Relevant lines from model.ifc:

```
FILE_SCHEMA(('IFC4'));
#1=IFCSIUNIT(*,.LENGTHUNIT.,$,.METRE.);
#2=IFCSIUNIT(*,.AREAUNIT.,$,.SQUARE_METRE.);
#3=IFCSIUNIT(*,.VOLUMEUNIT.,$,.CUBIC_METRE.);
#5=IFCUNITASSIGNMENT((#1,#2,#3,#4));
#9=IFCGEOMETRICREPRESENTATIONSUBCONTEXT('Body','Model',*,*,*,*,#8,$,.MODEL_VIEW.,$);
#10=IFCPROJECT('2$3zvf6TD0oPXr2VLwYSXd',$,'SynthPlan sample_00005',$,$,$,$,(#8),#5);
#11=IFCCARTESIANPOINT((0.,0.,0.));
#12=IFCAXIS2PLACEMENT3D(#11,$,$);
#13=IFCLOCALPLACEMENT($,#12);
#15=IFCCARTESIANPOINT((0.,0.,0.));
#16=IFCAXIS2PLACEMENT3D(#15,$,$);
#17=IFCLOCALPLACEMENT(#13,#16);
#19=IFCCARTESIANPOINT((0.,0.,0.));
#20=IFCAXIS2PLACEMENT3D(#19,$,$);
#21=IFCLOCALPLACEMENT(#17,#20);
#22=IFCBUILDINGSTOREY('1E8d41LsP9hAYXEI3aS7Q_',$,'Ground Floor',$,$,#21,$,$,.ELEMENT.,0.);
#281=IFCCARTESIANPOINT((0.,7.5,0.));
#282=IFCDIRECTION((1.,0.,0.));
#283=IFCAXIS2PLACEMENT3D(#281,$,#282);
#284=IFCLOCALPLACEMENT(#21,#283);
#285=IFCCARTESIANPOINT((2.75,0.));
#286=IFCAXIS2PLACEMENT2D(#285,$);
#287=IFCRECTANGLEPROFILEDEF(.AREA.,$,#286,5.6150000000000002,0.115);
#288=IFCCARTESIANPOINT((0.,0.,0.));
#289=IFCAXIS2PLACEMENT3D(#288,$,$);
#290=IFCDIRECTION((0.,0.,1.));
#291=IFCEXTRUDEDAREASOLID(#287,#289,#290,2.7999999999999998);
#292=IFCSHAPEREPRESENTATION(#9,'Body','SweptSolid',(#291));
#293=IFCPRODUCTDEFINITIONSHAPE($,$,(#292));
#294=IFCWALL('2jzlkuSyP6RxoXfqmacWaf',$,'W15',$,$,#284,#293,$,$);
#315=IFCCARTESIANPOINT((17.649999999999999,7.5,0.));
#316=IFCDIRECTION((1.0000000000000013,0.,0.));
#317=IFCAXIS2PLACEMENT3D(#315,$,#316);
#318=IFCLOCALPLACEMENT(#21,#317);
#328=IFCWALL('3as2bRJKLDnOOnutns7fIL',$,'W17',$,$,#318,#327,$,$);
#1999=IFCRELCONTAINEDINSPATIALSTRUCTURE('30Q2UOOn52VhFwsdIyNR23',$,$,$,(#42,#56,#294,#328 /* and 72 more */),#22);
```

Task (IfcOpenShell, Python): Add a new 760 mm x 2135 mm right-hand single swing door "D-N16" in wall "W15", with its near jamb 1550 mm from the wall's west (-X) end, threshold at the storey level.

```python
import numpy as np
import ifcopenshell
import ifcopenshell.api.feature
import ifcopenshell.api.geometry
import ifcopenshell.api.root
import ifcopenshell.api.spatial
import ifcopenshell.geom
import ifcopenshell.util.element
import ifcopenshell.util.placement
import ifcopenshell.util.representation
import ifcopenshell.util.shape
import ifcopenshell.util.unit

model = ifcopenshell.open("model.ifc")
unit_scale = ifcopenshell.util.unit.calculate_unit_scale(model)
settings = ifcopenshell.geom.settings()


def volume(element):
    """Net volume in cubic metres, openings subtracted."""
    shape = ifcopenshell.geom.create_shape(settings, element)
    return ifcopenshell.util.shape.get_volume(shape.geometry)


wall = model.by_guid("2jzlkuSyP6RxoXfqmacWaf")
storey = ifcopenshell.util.element.get_container(wall, ifc_class="IfcBuildingStorey")
context = ifcopenshell.util.representation.get_context(model, "Model", "Body", "MODEL_VIEW")
before = volume(wall)

width, height, from_end, sill = 0.76, 2.135, 1.55, 0.0  # metres

# The wall runs along its own X axis, and the end named is its -X end.
wall_shape = ifcopenshell.geom.create_shape(settings, wall)
x, y, z = ifcopenshell.util.shape.get_vertices(wall_shape.geometry).T
start = x.min() + from_end
face, thickness = float(y.min()), float(y.max() - y.min())
wall_matrix = ifcopenshell.util.placement.get_local_placement(wall.ObjectPlacement)
level = ifcopenshell.util.placement.get_local_placement(storey.ObjectPlacement)[2, 3]


def in_wall(x, y):
    """Placement at x, y metres in the wall's axes, at sill height."""
    matrix = wall_matrix.copy()
    matrix[:, 3] = wall_matrix @ np.array([x / unit_scale, y / unit_scale, 0.0, 1.0])
    matrix[2, 3] = level + sill / unit_scale
    return matrix


# Opening: a box that overshoots both wall faces by 50 mm.
opening = ifcopenshell.api.root.create_entity(model, ifc_class="IfcOpeningElement", predefined_type="OPENING")
box = ifcopenshell.api.geometry.add_wall_representation(
    model, context=context, length=width, height=height, thickness=thickness + 0.1
)
ifcopenshell.api.geometry.assign_representation(model, product=opening, representation=box)
ifcopenshell.api.geometry.edit_object_placement(model, product=opening, matrix=in_wall(start, face - 0.05), is_si=False)
ifcopenshell.api.feature.add_feature(model, feature=opening, element=wall)

door = ifcopenshell.api.root.create_entity(model, ifc_class="IfcDoor", name="D-N16", predefined_type="DOOR")
door.OverallWidth, door.OverallHeight = width / unit_scale, height / unit_scale
door.OperationType = "SINGLE_SWING_RIGHT"
body = ifcopenshell.api.geometry.add_door_representation(
    model,
    context=context,
    overall_width=door.OverallWidth,
    overall_height=door.OverallHeight,
    operation_type="SINGLE_SWING_RIGHT",
    lining_properties={"LiningDepth": thickness / unit_scale, "ThresholdDepth": thickness / unit_scale},
)
ifcopenshell.api.geometry.assign_representation(model, product=door, representation=body)
ifcopenshell.api.spatial.assign_container(model, products=[door], relating_structure=storey)
ifcopenshell.api.feature.add_filling(model, opening=opening, element=door)

# The lining spans the wall, so the door starts at the wall face.
ifcopenshell.api.geometry.edit_object_placement(model, product=door, matrix=in_wall(start, face), is_si=False)

after = volume(wall)

print(f"wall volume {before:.3f} -> {after:.3f} m3")

model.write("model_edited.ifc")
```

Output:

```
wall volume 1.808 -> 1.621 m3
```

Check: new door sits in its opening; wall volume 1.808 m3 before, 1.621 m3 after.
